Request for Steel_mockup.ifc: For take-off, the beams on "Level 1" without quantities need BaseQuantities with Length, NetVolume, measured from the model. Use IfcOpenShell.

First a look at what the model holds.

```python
import ifcopenshell
import ifcopenshell.util.element
import ifcopenshell.util.unit

model = ifcopenshell.open("Steel_mockup.ifc")
print(model.schema)
for unit_type in ("LENGTHUNIT", "AREAUNIT", "VOLUMEUNIT"):
    print(unit_type, ifcopenshell.util.unit.calculate_unit_scale(model, unit_type))
storey = next(s for s in model.by_type("IfcBuildingStorey") if s.Name == "Level 1")
beams = [e for e in ifcopenshell.util.element.get_decomposition(storey) if e.is_a("IfcBeam")]
for e in sorted(beams, key=lambda e: e.id()):
    print(e.id(), e.is_a(), e.Name, list(ifcopenshell.util.element.get_psets(e, qtos_only=True)), sep=" | ")
```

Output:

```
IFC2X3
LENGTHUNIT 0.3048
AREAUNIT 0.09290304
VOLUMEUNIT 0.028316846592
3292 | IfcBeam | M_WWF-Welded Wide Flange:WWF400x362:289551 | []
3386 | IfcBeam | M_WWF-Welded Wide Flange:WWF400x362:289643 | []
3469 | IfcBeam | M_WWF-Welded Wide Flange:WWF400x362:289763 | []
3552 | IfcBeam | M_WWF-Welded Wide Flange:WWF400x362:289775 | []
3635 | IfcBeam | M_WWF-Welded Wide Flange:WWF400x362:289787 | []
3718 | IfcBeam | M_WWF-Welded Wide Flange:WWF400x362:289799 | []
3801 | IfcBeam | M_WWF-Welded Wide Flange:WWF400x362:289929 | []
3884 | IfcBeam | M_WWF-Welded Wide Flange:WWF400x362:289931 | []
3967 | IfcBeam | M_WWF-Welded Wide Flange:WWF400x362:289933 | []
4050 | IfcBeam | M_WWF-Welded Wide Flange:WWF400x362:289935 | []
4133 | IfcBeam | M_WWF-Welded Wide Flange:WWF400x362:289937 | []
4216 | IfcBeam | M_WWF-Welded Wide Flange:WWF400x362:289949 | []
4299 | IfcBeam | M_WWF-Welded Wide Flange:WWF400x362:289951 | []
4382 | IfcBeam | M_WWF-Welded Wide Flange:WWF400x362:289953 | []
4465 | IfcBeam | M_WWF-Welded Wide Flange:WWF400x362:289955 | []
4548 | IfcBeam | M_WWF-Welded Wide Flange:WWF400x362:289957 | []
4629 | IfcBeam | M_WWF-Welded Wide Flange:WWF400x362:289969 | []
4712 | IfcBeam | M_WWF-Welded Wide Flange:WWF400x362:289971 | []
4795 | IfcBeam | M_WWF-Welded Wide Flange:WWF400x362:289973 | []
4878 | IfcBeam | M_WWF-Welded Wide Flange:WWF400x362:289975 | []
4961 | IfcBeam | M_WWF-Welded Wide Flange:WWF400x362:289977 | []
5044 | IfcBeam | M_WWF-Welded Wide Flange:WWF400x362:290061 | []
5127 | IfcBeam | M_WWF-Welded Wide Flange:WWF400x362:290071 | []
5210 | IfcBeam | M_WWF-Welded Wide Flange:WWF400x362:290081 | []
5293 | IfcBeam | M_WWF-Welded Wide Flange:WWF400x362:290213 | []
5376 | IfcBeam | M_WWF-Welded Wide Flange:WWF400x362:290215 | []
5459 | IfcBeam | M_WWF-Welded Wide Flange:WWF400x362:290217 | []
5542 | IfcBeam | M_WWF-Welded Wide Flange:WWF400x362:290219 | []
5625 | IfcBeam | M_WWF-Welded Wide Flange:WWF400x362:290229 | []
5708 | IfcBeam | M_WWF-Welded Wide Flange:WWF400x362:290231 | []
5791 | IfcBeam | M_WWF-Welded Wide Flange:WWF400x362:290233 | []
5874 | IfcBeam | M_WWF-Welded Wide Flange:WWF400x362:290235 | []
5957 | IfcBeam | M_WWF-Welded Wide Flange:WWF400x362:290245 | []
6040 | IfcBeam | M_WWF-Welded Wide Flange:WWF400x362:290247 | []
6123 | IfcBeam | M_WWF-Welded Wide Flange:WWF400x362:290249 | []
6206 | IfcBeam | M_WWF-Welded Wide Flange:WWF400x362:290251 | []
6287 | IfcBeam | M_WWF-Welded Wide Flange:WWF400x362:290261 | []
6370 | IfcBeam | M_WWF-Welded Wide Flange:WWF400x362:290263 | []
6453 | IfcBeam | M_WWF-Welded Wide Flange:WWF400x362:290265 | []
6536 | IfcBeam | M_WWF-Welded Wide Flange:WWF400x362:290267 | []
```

```python
import ifcopenshell
import ifcopenshell.api.pset
import ifcopenshell.geom
import ifcopenshell.util.element
import ifcopenshell.util.shape
import ifcopenshell.util.unit

model = ifcopenshell.open("Steel_mockup.ifc")
unit_scale = ifcopenshell.util.unit.calculate_unit_scale(model)
volume_scale = ifcopenshell.util.unit.calculate_unit_scale(model, "VOLUMEUNIT")
settings = ifcopenshell.geom.settings()

storey = next(s for s in model.by_type("IfcBuildingStorey") if s.Name == "Level 1")
beams = [e for e in ifcopenshell.util.element.get_decomposition(storey) if e.is_a("IfcBeam")]

for e in sorted(beams, key=lambda e: e.id()):
    if ifcopenshell.util.element.get_psets(e, qtos_only=True, should_inherit=False):
        continue
    # Geometry comes back in metres, in the element's own axes.
    shape = ifcopenshell.geom.create_shape(settings, e)
    values = {
        "Length": ifcopenshell.util.shape.get_max_xyz(shape.geometry) / unit_scale,
        "NetVolume": ifcopenshell.util.shape.get_volume(shape.geometry) / volume_scale,
    }
    qto = ifcopenshell.api.pset.add_qto(model, product=e, name="BaseQuantities")
    ifcopenshell.api.pset.edit_qto(model, qto=qto, properties=values)
    print(e.id(), {k: round(v, 3) for k, v in values.items()})

model.write("Steel_mockup_edited.ifc")
```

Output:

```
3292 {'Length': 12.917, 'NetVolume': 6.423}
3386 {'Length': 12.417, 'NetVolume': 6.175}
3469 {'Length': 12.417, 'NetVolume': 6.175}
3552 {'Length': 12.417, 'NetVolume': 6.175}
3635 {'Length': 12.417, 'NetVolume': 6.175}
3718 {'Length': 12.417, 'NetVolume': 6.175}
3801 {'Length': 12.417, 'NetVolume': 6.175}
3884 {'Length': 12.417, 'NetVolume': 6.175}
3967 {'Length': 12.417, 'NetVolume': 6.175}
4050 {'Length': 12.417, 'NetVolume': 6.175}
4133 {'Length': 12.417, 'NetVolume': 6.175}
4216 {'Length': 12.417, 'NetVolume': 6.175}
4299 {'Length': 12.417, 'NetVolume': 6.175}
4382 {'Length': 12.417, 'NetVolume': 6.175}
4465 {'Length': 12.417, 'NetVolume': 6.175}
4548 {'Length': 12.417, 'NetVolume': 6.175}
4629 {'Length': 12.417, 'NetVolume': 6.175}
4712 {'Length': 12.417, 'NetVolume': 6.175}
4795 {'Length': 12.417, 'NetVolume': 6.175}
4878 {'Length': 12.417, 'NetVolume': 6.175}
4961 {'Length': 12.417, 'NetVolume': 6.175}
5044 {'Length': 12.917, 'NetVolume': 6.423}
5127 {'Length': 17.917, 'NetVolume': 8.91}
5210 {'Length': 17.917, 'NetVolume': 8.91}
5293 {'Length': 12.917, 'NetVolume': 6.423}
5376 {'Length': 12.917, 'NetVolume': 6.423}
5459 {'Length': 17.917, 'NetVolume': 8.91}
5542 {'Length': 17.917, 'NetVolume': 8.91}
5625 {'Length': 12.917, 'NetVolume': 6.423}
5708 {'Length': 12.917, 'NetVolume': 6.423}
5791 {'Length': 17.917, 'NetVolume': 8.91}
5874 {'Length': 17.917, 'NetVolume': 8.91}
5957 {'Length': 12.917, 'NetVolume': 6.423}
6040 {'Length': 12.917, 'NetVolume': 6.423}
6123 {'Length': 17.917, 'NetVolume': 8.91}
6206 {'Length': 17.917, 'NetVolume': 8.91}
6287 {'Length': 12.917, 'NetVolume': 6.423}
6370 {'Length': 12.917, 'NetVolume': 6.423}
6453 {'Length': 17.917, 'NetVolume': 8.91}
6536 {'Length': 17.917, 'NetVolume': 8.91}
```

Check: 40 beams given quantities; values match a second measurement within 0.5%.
